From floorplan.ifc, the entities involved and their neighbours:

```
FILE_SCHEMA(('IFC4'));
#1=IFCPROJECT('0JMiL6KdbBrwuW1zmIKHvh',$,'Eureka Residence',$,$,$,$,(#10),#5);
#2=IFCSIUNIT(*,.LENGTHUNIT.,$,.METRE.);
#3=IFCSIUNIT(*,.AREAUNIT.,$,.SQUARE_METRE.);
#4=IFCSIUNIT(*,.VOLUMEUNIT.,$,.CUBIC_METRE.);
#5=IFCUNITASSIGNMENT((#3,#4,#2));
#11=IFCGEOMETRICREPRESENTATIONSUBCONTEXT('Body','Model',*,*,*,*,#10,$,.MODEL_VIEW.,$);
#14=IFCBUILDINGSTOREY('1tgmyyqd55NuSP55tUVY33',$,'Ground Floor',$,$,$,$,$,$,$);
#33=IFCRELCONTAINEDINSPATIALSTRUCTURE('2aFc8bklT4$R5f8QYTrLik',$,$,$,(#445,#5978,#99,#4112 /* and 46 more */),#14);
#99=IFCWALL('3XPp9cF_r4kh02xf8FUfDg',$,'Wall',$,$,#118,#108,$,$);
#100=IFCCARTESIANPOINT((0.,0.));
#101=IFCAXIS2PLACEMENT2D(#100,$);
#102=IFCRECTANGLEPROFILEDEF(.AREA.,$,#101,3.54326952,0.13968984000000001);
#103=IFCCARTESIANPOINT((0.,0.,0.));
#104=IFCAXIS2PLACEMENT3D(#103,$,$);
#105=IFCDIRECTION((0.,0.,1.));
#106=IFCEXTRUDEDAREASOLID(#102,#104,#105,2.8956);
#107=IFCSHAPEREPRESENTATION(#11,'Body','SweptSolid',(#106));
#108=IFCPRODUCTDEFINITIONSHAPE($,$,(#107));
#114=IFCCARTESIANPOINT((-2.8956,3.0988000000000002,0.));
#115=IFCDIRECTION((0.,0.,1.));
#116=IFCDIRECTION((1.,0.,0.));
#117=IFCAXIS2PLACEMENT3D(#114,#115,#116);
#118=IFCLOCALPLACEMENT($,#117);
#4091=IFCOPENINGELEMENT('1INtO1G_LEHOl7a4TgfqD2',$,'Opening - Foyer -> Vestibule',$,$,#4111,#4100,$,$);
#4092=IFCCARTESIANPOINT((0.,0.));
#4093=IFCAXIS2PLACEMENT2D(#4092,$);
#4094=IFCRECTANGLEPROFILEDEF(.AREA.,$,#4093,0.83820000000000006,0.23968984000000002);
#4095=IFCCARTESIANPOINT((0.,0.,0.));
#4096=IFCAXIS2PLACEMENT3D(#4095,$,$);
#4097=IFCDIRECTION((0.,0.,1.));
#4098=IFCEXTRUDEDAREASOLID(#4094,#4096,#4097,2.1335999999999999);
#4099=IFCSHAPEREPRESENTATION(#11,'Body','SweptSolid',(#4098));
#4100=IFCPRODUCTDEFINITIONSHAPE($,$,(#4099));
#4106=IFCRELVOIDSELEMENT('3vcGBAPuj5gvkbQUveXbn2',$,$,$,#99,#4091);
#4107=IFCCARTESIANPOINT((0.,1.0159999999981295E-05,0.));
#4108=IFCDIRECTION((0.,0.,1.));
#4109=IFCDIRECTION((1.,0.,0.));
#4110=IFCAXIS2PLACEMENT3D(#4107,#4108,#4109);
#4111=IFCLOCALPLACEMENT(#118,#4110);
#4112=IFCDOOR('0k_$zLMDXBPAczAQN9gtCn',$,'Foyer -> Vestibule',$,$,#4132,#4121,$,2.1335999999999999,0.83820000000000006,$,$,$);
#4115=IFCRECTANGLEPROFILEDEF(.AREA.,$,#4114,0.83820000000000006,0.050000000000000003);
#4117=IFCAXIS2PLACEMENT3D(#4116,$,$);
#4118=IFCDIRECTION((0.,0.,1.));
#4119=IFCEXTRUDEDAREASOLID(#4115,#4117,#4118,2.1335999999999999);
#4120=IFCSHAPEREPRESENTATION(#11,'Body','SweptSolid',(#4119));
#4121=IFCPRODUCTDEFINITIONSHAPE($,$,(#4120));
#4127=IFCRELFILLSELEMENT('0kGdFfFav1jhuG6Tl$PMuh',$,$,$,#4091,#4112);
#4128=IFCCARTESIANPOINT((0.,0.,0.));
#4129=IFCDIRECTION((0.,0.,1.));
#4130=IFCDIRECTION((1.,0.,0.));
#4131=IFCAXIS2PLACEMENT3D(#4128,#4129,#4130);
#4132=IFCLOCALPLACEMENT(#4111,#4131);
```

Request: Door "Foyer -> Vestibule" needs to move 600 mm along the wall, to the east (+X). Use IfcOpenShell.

```python
import ifcopenshell
import ifcopenshell.api.geometry
import ifcopenshell.util.placement
import ifcopenshell.util.unit

model = ifcopenshell.open("floorplan.ifc")
unit_scale = ifcopenshell.util.unit.calculate_unit_scale(model)

door = model.by_guid("0k_$zLMDXBPAczAQN9gtCn")
opening = door.FillsVoids[0].RelatingOpeningElement
wall = opening.VoidsElements[0].RelatingBuildingElement

wall_matrix = ifcopenshell.util.placement.get_local_placement(wall.ObjectPlacement)
shift = wall_matrix[:3, 0] * 0.6 / unit_scale
before = ifcopenshell.util.placement.get_local_placement(door.ObjectPlacement)[:3, 3].copy()

# The door is placed relative to its opening, so it follows when the opening moves.
matrix = ifcopenshell.util.placement.get_local_placement(opening.ObjectPlacement)
matrix[:3, 3] += shift
ifcopenshell.api.geometry.edit_object_placement(
    model, product=opening, matrix=matrix, is_si=False, should_transform_children=True
)

after = ifcopenshell.util.placement.get_local_placement(door.ObjectPlacement)[:3, 3]
print("door moved by", (after - before).round(3) + 0.0)

model.write("floorplan_v2.ifc")
```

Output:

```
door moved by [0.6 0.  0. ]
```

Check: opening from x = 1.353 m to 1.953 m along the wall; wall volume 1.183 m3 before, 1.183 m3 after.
